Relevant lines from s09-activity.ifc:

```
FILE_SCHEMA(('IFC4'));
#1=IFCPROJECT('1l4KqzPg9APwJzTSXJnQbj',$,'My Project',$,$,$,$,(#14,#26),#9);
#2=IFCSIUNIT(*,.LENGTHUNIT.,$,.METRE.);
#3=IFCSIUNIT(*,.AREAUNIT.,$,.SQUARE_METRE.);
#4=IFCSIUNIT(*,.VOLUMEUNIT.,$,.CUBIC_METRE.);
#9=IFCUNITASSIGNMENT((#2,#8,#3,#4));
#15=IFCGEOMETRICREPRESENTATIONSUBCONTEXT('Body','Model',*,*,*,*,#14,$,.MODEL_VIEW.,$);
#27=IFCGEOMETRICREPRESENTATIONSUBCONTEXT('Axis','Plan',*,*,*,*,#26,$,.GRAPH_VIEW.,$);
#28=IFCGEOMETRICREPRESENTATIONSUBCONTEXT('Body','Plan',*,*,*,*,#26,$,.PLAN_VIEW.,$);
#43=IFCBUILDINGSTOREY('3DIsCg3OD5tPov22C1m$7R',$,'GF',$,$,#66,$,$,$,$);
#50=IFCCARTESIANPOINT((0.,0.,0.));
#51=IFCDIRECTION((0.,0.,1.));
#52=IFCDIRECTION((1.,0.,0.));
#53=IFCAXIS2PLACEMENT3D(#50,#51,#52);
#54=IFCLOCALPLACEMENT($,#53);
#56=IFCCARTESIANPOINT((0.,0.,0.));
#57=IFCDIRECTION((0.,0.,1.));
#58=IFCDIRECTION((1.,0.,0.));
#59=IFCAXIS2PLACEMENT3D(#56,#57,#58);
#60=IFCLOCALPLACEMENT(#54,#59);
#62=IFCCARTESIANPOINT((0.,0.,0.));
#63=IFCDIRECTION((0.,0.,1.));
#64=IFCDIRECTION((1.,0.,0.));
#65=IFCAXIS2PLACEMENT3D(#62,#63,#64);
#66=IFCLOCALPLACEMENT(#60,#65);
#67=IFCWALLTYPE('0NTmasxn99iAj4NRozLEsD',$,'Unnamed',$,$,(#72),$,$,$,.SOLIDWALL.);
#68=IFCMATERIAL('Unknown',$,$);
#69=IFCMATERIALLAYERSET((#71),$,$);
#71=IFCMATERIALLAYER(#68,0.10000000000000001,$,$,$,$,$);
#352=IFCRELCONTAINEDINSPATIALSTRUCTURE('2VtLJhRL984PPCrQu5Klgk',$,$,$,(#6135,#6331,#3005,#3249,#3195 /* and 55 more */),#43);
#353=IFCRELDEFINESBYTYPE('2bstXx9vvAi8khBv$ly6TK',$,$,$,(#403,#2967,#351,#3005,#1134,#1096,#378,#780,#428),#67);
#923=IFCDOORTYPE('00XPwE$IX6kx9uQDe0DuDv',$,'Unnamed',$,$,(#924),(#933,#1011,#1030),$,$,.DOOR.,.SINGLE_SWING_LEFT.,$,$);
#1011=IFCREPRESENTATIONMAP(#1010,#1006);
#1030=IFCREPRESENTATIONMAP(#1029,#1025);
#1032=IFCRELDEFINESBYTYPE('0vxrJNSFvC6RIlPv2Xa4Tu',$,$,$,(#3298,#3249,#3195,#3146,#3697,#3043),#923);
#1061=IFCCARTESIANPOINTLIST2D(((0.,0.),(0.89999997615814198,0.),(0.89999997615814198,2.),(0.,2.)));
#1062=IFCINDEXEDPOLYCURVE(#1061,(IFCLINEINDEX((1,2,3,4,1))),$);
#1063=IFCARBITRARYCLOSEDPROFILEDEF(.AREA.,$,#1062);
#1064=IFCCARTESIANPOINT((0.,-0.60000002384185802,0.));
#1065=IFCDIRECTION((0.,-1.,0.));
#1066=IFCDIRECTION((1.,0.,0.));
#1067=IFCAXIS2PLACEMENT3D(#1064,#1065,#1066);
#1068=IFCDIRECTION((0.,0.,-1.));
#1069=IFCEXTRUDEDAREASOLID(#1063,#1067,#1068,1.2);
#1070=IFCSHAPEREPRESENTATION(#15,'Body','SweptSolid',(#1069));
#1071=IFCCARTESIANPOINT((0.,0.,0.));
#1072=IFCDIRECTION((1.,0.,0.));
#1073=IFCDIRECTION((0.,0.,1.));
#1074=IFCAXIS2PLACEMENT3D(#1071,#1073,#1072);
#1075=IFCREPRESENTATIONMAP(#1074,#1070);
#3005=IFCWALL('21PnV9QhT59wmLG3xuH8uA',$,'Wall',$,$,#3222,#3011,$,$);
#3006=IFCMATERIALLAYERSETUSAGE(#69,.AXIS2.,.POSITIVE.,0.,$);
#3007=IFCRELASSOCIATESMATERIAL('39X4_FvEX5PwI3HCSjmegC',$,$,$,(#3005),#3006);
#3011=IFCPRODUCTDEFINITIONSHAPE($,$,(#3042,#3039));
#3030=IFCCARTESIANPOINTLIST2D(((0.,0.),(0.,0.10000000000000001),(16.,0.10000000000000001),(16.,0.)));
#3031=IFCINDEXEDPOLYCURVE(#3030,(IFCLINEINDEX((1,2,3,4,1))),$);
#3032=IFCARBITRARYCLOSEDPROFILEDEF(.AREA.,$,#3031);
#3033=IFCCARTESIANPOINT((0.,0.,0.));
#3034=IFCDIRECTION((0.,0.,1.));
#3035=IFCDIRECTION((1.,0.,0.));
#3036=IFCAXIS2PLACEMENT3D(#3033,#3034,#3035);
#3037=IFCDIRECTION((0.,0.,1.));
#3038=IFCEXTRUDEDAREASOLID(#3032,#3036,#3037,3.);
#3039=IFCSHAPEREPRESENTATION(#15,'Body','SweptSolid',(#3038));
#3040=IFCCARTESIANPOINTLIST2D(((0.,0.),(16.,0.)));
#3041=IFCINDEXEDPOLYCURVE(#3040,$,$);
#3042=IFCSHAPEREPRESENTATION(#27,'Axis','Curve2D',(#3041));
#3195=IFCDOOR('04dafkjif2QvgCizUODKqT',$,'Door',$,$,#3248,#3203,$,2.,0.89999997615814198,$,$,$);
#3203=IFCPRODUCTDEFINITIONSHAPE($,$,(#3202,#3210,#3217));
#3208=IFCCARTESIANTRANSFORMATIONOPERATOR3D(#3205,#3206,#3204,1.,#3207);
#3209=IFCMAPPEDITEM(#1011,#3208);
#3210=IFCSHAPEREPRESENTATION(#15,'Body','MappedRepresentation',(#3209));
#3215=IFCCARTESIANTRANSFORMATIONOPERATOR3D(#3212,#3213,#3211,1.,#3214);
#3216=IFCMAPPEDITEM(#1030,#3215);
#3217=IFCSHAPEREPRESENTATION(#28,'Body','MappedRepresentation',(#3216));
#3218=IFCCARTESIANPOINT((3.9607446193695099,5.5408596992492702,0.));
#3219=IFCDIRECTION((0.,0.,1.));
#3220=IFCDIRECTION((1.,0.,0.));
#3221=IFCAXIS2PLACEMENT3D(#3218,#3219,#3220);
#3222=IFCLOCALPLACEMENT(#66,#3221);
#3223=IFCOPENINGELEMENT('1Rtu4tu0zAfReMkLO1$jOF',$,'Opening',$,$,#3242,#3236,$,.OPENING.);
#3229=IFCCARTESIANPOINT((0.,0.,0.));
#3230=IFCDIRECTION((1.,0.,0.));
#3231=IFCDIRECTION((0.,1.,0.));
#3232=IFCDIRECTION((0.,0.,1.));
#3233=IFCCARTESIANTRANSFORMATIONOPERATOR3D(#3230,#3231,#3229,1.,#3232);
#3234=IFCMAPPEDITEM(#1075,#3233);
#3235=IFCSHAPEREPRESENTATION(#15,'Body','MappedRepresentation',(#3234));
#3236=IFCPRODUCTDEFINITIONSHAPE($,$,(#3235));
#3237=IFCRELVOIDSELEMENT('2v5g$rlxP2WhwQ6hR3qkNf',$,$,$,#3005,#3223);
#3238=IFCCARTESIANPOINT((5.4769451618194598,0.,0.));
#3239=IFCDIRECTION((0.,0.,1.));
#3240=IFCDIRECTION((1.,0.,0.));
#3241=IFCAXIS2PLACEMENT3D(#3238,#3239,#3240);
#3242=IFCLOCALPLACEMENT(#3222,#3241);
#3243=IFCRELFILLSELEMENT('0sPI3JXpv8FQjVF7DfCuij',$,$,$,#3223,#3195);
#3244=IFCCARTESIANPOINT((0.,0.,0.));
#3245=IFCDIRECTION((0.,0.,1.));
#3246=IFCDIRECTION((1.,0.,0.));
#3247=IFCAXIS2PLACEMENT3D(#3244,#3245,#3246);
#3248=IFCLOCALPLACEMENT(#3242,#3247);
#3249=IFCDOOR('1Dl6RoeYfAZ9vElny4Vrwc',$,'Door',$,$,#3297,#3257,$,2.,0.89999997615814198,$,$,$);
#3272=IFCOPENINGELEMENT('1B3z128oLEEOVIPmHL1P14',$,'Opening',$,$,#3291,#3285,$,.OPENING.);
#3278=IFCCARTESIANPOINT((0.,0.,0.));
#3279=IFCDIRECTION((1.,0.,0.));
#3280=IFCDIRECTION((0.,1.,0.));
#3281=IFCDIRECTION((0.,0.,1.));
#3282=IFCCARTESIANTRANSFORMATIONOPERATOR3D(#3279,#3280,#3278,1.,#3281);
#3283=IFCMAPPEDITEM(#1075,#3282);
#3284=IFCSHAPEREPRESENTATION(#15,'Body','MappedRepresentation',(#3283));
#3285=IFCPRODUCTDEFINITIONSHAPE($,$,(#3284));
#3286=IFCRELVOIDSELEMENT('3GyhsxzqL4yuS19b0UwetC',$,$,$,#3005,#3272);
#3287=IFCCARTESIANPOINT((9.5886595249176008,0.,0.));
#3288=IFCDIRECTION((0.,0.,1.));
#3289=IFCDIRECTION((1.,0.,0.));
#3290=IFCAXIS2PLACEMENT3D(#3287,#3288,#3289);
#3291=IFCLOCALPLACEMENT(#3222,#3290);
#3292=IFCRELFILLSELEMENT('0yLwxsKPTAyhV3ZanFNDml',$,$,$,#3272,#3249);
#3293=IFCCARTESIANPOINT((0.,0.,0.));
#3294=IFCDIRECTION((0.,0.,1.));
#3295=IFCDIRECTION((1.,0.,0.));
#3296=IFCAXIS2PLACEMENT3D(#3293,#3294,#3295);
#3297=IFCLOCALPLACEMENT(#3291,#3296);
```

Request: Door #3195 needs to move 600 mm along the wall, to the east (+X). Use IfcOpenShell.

```python
import ifcopenshell
import ifcopenshell.api.geometry
import ifcopenshell.util.placement
import ifcopenshell.util.unit

model = ifcopenshell.open("s09-activity.ifc")
unit_scale = ifcopenshell.util.unit.calculate_unit_scale(model)

door = model.by_guid("04dafkjif2QvgCizUODKqT")
opening = door.FillsVoids[0].RelatingOpeningElement
wall = opening.VoidsElements[0].RelatingBuildingElement

wall_matrix = ifcopenshell.util.placement.get_local_placement(wall.ObjectPlacement)
shift = wall_matrix[:3, 0] * 0.6 / unit_scale
before = ifcopenshell.util.placement.get_local_placement(door.ObjectPlacement)[:3, 3].copy()

# The door is placed relative to its opening, so it follows when the opening moves.
matrix = ifcopenshell.util.placement.get_local_placement(opening.ObjectPlacement)
matrix[:3, 3] += shift
ifcopenshell.api.geometry.edit_object_placement(
    model, product=opening, matrix=matrix, is_si=False, should_transform_children=True
)

after = ifcopenshell.util.placement.get_local_placement(door.ObjectPlacement)[:3, 3]
print("door moved by", (after - before).round(3) + 0.0)

model.write("s09-activity_edited.ifc")
```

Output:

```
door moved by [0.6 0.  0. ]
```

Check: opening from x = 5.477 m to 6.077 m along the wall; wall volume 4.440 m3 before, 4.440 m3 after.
